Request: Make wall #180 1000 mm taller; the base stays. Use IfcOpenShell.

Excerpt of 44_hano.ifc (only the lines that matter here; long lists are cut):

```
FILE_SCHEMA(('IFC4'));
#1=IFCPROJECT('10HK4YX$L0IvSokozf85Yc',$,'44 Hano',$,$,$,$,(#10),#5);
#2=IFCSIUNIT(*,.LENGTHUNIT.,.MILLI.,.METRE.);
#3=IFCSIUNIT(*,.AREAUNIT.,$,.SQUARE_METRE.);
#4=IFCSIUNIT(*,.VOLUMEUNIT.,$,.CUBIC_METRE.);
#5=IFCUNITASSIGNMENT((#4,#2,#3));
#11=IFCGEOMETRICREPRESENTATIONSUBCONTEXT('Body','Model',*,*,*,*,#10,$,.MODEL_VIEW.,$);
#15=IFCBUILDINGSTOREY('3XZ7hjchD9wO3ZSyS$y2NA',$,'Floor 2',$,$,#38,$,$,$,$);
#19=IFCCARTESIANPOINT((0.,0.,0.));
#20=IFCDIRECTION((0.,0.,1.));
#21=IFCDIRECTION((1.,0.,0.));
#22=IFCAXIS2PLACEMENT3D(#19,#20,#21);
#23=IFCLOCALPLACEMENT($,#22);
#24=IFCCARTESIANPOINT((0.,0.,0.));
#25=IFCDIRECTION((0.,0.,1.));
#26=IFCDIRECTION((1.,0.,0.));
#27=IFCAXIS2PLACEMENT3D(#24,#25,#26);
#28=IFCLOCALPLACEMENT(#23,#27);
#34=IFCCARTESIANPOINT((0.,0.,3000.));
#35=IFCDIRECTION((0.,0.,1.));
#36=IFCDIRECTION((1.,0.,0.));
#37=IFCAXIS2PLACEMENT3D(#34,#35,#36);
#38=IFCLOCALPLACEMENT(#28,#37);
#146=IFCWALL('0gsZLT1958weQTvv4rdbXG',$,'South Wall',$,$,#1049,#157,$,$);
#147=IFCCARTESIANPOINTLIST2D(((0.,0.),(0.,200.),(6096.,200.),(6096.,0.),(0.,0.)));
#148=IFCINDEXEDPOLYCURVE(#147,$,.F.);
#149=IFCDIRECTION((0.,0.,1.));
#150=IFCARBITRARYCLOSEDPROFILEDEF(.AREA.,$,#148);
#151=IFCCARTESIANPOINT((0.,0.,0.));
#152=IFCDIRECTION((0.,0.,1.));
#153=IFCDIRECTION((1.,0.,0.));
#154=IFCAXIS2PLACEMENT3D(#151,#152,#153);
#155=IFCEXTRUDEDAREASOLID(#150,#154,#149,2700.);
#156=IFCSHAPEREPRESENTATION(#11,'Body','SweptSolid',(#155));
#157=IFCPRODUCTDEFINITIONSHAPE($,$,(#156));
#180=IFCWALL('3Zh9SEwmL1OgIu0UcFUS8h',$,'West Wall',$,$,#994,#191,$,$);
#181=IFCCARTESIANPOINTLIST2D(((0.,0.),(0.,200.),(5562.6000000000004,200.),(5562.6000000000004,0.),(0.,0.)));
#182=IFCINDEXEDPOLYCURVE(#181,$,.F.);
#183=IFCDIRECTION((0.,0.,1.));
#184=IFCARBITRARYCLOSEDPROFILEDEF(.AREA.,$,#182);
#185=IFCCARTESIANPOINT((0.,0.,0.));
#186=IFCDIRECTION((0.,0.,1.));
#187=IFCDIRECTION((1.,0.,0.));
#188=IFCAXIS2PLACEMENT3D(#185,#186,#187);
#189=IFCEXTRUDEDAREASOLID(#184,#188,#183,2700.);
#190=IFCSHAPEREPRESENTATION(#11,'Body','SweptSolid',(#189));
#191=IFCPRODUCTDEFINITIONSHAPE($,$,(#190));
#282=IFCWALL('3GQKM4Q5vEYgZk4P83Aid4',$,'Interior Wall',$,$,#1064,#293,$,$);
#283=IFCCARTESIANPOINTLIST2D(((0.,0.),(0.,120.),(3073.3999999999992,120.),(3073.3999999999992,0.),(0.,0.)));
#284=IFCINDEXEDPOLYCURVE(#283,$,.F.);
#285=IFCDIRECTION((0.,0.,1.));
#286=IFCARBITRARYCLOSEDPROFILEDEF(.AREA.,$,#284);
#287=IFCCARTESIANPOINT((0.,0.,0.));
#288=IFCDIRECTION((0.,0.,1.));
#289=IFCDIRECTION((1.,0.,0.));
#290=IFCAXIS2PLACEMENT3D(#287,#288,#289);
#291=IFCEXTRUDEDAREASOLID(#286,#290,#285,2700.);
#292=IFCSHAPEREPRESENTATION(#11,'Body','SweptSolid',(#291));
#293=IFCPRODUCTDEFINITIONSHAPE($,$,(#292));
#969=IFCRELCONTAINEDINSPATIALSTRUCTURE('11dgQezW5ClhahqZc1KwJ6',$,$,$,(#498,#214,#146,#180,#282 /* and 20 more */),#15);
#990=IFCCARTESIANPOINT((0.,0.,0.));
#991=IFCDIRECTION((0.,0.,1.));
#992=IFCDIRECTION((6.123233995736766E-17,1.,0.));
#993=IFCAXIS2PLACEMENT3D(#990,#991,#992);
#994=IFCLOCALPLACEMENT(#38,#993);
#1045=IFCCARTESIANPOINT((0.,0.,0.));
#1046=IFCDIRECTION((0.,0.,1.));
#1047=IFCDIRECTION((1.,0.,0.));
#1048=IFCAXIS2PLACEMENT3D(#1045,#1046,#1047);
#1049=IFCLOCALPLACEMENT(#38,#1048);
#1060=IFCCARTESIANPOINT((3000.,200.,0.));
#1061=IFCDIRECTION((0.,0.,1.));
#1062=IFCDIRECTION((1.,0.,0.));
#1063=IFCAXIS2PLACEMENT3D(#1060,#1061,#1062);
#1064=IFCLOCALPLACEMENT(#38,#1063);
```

```python
import ifcopenshell
import ifcopenshell.geom
import ifcopenshell.util.representation
import ifcopenshell.util.shape
import ifcopenshell.util.unit

model = ifcopenshell.open("44_hano.ifc")
unit_scale = ifcopenshell.util.unit.calculate_unit_scale(model)
settings = ifcopenshell.geom.settings()


def volume(element):
    """Net volume in cubic metres, openings subtracted."""
    shape = ifcopenshell.geom.create_shape(settings, element)
    return ifcopenshell.util.shape.get_volume(shape.geometry)


wall = model.by_guid("3Zh9SEwmL1OgIu0UcFUS8h")
before = volume(wall)

body = ifcopenshell.util.representation.get_representation(wall, "Model", "Body")
solid = body.Items[0]
old_height = solid.Depth
solid.Depth += 1 / unit_scale
after = volume(wall)

print(f"height {old_height:g} -> {solid.Depth:g}, volume {before:.3f} -> {after:.3f} m3")

model.write("44_hano-out.ifc")
```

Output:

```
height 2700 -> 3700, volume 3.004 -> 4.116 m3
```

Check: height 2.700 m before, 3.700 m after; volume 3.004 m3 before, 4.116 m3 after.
